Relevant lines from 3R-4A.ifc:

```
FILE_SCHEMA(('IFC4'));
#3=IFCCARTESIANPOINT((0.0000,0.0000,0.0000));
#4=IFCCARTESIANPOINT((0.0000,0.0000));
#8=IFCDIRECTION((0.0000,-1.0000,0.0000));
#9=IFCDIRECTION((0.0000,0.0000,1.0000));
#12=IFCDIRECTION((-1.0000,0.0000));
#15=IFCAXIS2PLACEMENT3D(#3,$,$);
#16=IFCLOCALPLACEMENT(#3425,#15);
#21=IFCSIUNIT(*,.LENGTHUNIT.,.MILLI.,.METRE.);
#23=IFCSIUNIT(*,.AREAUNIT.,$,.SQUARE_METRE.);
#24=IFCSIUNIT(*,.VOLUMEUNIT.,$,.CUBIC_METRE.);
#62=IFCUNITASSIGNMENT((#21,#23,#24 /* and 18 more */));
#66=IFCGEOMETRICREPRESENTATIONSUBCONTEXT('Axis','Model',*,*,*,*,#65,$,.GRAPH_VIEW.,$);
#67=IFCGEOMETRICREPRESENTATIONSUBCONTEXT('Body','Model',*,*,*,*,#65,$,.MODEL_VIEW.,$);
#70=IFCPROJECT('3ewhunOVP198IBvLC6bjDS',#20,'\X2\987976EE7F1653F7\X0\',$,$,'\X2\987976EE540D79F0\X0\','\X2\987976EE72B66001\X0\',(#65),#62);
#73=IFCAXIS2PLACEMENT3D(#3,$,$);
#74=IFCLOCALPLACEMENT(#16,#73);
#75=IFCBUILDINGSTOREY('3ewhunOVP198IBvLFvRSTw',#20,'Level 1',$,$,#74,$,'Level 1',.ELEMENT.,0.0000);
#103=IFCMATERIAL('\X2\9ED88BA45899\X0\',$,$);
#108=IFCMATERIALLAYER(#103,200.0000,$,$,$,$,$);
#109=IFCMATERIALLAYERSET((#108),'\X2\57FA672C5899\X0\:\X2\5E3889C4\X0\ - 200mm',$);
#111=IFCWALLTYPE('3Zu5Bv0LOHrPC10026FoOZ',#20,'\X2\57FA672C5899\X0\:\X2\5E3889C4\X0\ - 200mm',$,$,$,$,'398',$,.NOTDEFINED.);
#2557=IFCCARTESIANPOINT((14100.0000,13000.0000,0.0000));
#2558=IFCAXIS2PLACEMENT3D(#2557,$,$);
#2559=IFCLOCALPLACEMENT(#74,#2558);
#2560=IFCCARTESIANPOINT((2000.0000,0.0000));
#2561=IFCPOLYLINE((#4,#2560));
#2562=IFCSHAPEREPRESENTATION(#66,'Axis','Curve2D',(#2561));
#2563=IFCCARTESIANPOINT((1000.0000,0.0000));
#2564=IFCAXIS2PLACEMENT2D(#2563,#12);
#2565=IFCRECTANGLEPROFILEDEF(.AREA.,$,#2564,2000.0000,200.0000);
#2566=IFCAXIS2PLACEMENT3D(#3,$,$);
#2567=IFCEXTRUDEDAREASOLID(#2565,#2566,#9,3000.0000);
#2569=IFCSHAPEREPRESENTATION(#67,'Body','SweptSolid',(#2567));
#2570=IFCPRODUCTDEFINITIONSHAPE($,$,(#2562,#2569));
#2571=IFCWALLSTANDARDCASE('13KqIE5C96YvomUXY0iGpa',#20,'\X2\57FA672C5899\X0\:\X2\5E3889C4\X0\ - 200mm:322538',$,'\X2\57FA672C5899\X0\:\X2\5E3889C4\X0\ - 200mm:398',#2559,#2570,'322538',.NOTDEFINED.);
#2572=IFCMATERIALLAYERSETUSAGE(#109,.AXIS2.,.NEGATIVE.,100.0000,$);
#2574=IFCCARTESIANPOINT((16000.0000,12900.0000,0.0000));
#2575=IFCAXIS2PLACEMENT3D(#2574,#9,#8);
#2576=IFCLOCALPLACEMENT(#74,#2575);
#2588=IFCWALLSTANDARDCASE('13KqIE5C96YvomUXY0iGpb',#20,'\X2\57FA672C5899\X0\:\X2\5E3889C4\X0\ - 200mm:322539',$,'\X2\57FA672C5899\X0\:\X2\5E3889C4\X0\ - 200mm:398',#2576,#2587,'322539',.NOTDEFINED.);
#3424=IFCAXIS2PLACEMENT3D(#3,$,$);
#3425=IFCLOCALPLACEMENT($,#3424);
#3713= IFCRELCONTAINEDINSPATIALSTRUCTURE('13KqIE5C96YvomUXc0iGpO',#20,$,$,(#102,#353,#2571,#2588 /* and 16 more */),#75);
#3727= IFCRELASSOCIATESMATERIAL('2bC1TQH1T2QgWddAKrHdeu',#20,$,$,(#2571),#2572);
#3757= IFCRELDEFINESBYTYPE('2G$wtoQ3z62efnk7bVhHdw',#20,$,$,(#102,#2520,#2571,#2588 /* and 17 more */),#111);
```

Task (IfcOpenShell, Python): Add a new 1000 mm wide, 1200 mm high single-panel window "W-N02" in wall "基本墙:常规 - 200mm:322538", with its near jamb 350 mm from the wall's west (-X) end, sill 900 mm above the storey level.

```python
import numpy as np
import ifcopenshell
import ifcopenshell.api.feature
import ifcopenshell.api.geometry
import ifcopenshell.api.root
import ifcopenshell.api.spatial
import ifcopenshell.geom
import ifcopenshell.util.element
import ifcopenshell.util.placement
import ifcopenshell.util.representation
import ifcopenshell.util.shape
import ifcopenshell.util.unit

model = ifcopenshell.open("3R-4A.ifc")
unit_scale = ifcopenshell.util.unit.calculate_unit_scale(model)
settings = ifcopenshell.geom.settings()


def volume(element):
    """Net volume in cubic metres, openings subtracted."""
    shape = ifcopenshell.geom.create_shape(settings, element)
    return ifcopenshell.util.shape.get_volume(shape.geometry)


wall = model.by_guid("13KqIE5C96YvomUXY0iGpa")
storey = ifcopenshell.util.element.get_container(wall, ifc_class="IfcBuildingStorey")
context = ifcopenshell.util.representation.get_context(model, "Model", "Body", "MODEL_VIEW")
before = volume(wall)

width, height, from_end, sill = 1, 1.2, 0.35, 0.9  # metres

# The wall runs along its own X axis, and the end named is its -X end.
wall_shape = ifcopenshell.geom.create_shape(settings, wall)
x, y, z = ifcopenshell.util.shape.get_vertices(wall_shape.geometry).T
start = x.min() + from_end
face, thickness = float(y.min()), float(y.max() - y.min())
wall_matrix = ifcopenshell.util.placement.get_local_placement(wall.ObjectPlacement)
level = ifcopenshell.util.placement.get_local_placement(storey.ObjectPlacement)[2, 3]


def in_wall(x, y):
    """Placement at x, y metres in the wall's axes, at sill height."""
    matrix = wall_matrix.copy()
    matrix[:, 3] = wall_matrix @ np.array([x / unit_scale, y / unit_scale, 0.0, 1.0])
    matrix[2, 3] = level + sill / unit_scale
    return matrix


# Opening: a box that overshoots both wall faces by 50 mm.
opening = ifcopenshell.api.root.create_entity(model, ifc_class="IfcOpeningElement", predefined_type="OPENING")
box = ifcopenshell.api.geometry.add_wall_representation(
    model, context=context, length=width, height=height, thickness=thickness + 0.1
)
ifcopenshell.api.geometry.assign_representation(model, product=opening, representation=box)
ifcopenshell.api.geometry.edit_object_placement(model, product=opening, matrix=in_wall(start, face - 0.05), is_si=False)
ifcopenshell.api.feature.add_feature(model, feature=opening, element=wall)

window = ifcopenshell.api.root.create_entity(model, ifc_class="IfcWindow", name="W-N02", predefined_type="WINDOW")
window.OverallWidth, window.OverallHeight = width / unit_scale, height / unit_scale
window.PartitioningType = "SINGLE_PANEL"
body = ifcopenshell.api.geometry.add_window_representation(
    model,
    context=context,
    overall_width=window.OverallWidth,
    overall_height=window.OverallHeight,
    partition_type="SINGLE_PANEL",
)
ifcopenshell.api.geometry.assign_representation(model, product=window, representation=body)
ifcopenshell.api.spatial.assign_container(model, products=[window], relating_structure=storey)
ifcopenshell.api.feature.add_filling(model, opening=opening, element=window)

# Centre the window in the wall's thickness.
ifcopenshell.api.geometry.edit_object_placement(model, product=window, matrix=in_wall(start, face), is_si=False)
window_shape = ifcopenshell.geom.create_shape(settings, window)
depth = ifcopenshell.util.shape.get_vertices(window_shape.geometry)[:, 1]
offset = face + thickness / 2 - (depth.min() + depth.max()) / 2
ifcopenshell.api.geometry.edit_object_placement(model, product=window, matrix=in_wall(start, offset), is_si=False)

after = volume(wall)

print(f"wall volume {before:.3f} -> {after:.3f} m3")

model.write("3R-4A_edited.ifc")
```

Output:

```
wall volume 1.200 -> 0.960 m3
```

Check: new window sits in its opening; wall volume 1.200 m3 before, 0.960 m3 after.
